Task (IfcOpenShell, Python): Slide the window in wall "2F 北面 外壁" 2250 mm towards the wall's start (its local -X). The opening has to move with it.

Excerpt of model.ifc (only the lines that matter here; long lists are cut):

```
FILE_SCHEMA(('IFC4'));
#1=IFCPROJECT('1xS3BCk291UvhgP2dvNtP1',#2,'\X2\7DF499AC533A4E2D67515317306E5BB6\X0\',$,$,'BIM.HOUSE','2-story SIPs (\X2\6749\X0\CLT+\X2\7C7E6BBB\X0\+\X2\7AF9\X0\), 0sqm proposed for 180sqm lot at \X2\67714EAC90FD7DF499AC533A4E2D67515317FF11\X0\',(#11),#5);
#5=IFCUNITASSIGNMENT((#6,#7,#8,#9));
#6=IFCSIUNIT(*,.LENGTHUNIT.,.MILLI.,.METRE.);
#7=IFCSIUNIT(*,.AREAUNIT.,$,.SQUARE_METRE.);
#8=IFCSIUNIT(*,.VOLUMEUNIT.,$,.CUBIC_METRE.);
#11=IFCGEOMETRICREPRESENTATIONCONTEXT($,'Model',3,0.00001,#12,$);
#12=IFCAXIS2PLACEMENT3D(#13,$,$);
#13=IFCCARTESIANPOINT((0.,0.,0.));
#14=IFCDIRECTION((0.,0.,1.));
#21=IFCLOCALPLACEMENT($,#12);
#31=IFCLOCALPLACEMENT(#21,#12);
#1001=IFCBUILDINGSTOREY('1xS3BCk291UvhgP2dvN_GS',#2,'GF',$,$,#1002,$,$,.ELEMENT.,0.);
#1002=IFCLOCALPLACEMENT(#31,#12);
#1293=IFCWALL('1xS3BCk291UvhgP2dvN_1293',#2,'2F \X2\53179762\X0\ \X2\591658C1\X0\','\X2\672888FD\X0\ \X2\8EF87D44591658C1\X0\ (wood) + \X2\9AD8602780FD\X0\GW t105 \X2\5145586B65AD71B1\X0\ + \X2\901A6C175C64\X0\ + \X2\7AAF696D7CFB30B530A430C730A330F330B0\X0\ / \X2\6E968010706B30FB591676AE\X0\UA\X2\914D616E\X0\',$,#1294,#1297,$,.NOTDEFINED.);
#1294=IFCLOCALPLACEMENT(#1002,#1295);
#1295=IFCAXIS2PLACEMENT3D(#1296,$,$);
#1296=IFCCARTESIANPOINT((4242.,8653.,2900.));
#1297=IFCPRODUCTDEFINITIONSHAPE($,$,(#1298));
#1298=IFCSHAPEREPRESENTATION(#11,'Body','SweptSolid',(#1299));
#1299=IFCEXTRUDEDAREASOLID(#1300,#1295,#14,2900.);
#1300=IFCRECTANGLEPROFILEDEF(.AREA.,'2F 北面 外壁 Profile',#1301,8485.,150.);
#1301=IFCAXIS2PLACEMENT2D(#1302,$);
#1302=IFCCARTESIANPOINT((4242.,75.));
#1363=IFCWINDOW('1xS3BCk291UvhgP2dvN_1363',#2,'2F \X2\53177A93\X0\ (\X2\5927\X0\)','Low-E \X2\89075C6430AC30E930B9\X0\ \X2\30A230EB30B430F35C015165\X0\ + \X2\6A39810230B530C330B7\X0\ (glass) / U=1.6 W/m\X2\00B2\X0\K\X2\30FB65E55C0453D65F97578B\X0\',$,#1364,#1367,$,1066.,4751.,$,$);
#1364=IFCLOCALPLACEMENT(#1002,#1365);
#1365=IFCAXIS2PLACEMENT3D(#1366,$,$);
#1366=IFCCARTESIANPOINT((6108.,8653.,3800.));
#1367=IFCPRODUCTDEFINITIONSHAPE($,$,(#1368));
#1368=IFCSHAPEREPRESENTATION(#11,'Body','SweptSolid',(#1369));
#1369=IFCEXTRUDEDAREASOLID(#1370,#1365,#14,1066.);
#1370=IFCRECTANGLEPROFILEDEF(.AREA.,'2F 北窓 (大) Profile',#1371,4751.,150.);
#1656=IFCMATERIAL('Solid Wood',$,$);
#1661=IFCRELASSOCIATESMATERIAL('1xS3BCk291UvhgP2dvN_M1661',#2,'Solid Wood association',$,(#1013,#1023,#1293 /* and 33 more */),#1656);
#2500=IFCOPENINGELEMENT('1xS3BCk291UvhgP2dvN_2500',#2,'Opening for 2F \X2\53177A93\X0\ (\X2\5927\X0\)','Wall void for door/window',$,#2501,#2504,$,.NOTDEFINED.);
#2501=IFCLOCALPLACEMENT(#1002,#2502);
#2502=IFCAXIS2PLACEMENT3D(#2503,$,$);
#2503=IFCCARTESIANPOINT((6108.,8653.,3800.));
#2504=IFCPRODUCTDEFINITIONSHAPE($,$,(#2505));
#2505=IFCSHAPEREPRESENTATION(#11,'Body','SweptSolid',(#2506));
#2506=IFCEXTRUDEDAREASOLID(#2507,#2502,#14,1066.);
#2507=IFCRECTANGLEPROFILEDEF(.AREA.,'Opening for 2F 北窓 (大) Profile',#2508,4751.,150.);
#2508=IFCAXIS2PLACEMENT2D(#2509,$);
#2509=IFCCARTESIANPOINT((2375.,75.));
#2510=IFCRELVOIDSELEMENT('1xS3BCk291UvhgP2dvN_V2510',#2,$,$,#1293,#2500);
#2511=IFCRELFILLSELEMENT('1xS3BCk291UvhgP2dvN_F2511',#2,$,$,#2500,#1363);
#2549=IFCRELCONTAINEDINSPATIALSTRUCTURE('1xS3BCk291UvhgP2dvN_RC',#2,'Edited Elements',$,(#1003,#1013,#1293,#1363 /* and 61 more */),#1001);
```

```python
import ifcopenshell
import ifcopenshell.api.geometry
import ifcopenshell.util.placement
import ifcopenshell.util.unit

model = ifcopenshell.open("model.ifc")
unit_scale = ifcopenshell.util.unit.calculate_unit_scale(model)

window = model.by_id(1363)
opening = window.FillsVoids[0].RelatingOpeningElement
wall = opening.VoidsElements[0].RelatingBuildingElement

wall_matrix = ifcopenshell.util.placement.get_local_placement(wall.ObjectPlacement)
shift = wall_matrix[:3, 0] * -2.25 / unit_scale
before = ifcopenshell.util.placement.get_local_placement(window.ObjectPlacement)[:3, 3].copy()

# The window is not placed relative to its opening, so move both.
for product in (opening, window):
    matrix = ifcopenshell.util.placement.get_local_placement(product.ObjectPlacement)
    matrix[:3, 3] += shift
    ifcopenshell.api.geometry.edit_object_placement(model, product=product, matrix=matrix, is_si=False)

after = ifcopenshell.util.placement.get_local_placement(window.ObjectPlacement)[:3, 3]
print("window moved by", (after - before).round(3) + 0.0)

model.write("model_v2.ifc")
```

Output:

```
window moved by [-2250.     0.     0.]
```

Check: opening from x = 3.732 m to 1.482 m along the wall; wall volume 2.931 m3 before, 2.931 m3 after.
